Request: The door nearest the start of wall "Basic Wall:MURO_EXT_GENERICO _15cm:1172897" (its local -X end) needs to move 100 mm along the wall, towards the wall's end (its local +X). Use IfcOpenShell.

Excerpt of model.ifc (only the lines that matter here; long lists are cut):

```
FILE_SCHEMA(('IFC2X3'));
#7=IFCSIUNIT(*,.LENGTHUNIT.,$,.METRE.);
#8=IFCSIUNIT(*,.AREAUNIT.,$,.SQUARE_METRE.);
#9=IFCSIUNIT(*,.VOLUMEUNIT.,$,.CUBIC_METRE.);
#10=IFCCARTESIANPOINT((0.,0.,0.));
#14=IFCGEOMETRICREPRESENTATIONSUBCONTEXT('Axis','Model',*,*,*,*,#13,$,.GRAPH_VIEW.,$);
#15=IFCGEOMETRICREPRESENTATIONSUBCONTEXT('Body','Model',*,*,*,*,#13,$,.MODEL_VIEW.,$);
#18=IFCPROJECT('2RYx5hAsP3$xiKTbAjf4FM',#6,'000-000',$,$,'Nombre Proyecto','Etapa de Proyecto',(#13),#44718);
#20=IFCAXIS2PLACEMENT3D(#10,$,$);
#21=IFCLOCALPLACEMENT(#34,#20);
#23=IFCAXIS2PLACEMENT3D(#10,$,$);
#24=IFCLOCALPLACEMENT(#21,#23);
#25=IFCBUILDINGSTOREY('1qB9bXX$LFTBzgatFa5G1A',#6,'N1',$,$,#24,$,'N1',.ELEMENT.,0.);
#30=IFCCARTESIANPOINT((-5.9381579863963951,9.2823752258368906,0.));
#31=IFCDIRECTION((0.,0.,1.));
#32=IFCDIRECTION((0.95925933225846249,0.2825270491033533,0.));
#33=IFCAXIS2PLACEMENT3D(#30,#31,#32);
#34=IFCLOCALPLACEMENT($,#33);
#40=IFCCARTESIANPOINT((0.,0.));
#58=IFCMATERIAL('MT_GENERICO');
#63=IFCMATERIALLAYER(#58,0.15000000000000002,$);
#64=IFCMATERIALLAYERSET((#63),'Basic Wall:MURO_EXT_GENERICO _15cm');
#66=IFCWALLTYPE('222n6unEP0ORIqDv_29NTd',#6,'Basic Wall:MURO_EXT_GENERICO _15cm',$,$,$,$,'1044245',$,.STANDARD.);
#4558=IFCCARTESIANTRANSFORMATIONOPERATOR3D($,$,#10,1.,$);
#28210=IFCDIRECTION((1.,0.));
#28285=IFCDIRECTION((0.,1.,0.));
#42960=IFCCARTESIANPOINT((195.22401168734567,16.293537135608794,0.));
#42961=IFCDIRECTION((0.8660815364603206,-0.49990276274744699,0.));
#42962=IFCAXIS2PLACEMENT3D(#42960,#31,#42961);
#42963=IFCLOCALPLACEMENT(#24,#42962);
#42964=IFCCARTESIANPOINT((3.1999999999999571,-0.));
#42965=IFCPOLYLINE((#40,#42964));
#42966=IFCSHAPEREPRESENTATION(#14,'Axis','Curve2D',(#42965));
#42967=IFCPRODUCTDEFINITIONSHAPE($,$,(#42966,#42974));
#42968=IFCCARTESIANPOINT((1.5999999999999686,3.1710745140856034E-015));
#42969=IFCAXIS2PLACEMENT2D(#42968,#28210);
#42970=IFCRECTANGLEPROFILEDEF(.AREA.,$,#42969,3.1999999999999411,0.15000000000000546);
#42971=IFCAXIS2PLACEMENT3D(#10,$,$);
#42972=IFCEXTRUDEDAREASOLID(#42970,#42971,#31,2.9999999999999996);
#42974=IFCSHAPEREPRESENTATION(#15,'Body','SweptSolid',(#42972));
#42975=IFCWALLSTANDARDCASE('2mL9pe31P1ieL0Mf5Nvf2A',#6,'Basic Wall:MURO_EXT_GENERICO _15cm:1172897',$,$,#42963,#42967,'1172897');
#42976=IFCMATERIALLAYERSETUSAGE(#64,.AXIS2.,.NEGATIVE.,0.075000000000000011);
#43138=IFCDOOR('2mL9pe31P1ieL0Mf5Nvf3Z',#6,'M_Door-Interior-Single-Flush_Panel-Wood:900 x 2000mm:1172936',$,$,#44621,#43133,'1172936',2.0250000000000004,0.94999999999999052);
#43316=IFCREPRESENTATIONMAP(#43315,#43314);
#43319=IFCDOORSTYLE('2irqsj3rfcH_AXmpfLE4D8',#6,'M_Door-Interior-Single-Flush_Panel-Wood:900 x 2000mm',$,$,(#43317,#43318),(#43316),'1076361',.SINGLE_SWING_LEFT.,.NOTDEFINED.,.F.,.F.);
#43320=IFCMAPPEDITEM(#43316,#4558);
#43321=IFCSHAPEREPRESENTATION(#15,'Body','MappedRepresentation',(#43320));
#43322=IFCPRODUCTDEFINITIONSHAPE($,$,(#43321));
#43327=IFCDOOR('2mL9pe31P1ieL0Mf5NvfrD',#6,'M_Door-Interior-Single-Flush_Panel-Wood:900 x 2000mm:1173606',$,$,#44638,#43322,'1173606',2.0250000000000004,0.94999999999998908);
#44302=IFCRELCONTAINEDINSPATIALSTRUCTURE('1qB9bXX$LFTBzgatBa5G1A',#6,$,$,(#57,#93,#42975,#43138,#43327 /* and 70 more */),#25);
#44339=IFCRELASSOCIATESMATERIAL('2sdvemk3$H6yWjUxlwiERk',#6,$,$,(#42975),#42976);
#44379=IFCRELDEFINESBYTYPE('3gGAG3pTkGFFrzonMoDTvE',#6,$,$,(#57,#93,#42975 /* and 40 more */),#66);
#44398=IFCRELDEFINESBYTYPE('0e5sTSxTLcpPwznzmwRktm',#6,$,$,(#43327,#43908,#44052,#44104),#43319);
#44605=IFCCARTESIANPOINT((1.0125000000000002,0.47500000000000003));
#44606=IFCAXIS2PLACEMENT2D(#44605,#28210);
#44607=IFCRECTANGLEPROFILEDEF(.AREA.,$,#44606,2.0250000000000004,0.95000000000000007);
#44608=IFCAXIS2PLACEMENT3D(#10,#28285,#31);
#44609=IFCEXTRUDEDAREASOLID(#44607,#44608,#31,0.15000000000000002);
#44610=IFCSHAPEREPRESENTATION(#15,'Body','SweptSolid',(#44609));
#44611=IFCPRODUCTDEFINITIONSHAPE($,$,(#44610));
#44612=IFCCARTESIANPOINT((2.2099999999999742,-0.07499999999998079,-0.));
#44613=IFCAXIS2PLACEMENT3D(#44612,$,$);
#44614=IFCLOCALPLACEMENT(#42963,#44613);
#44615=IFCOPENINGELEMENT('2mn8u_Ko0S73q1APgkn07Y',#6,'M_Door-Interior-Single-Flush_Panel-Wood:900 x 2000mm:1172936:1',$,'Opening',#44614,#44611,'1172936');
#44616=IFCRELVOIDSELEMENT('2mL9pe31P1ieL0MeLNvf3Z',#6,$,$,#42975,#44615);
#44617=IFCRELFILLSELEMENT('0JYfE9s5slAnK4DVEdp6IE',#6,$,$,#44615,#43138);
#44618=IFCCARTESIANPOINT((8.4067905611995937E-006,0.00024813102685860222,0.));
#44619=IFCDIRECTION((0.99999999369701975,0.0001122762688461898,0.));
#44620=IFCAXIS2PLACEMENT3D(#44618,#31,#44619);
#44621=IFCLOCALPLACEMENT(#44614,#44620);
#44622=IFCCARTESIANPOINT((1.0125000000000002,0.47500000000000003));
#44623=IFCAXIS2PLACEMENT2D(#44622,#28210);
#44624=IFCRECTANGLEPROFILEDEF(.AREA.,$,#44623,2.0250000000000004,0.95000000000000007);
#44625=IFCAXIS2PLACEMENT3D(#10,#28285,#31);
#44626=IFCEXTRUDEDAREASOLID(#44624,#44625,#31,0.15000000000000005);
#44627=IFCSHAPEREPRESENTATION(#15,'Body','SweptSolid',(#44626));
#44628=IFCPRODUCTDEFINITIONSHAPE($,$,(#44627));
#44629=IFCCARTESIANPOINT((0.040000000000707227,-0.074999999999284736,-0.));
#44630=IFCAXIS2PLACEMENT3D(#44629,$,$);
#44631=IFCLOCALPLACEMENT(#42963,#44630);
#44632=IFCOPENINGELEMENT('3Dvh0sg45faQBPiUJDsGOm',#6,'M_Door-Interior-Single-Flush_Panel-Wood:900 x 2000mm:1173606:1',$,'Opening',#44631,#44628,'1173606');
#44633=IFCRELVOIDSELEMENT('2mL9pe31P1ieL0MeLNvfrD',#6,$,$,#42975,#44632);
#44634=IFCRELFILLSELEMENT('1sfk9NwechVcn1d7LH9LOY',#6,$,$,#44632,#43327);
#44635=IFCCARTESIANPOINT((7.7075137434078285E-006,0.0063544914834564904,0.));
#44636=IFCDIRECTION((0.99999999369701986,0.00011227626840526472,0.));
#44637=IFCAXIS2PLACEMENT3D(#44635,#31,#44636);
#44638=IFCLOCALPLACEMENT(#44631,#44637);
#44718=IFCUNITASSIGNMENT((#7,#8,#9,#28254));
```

```python
import ifcopenshell
import ifcopenshell.api.geometry
import ifcopenshell.util.placement

model = ifcopenshell.open("model.ifc")

door = model.by_guid("2mL9pe31P1ieL0Mf5NvfrD")
opening = door.FillsVoids[0].RelatingOpeningElement
wall = opening.VoidsElements[0].RelatingBuildingElement

wall_matrix = ifcopenshell.util.placement.get_local_placement(wall.ObjectPlacement)
shift = wall_matrix[:3, 0] * 0.1
before = ifcopenshell.util.placement.get_local_placement(door.ObjectPlacement)[:3, 3].copy()

# The door is placed relative to its opening, so it follows when the opening moves.
matrix = ifcopenshell.util.placement.get_local_placement(opening.ObjectPlacement)
matrix[:3, 3] += shift
ifcopenshell.api.geometry.edit_object_placement(
    model, product=opening, matrix=matrix, is_si=False, should_transform_children=True
)

after = ifcopenshell.util.placement.get_local_placement(door.ObjectPlacement)[:3, 3]
print("door moved by", (after - before).round(3) + 0.0)

model.write("model-out.ifc")
```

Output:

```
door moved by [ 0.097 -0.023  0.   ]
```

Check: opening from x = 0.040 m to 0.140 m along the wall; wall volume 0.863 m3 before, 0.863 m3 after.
